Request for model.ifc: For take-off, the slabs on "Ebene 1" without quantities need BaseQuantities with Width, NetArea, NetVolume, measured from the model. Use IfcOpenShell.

First a look at what the model holds.

```python
import ifcopenshell
import ifcopenshell.util.element
import ifcopenshell.util.unit

model = ifcopenshell.open("model.ifc")
print(model.schema)
for unit_type in ("LENGTHUNIT", "AREAUNIT", "VOLUMEUNIT"):
    print(unit_type, ifcopenshell.util.unit.calculate_unit_scale(model, unit_type))
storey = next(s for s in model.by_type("IfcBuildingStorey") if s.Name == "Ebene 1")
slabs = [e for e in ifcopenshell.util.element.get_decomposition(storey) if e.is_a("IfcSlab")]
for e in sorted(slabs, key=lambda e: e.id()):
    print(e.id(), e.is_a(), e.Name, list(ifcopenshell.util.element.get_psets(e, qtos_only=True)), sep=" | ")
```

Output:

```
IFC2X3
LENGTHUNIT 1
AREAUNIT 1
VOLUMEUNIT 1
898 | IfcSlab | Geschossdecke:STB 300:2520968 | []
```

```python
import ifcopenshell
import ifcopenshell.api.pset
import ifcopenshell.geom
import ifcopenshell.util.element
import ifcopenshell.util.shape
import ifcopenshell.util.unit

model = ifcopenshell.open("model.ifc")
unit_scale = ifcopenshell.util.unit.calculate_unit_scale(model)
area_scale = ifcopenshell.util.unit.calculate_unit_scale(model, "AREAUNIT")
volume_scale = ifcopenshell.util.unit.calculate_unit_scale(model, "VOLUMEUNIT")
settings = ifcopenshell.geom.settings()

storey = next(s for s in model.by_type("IfcBuildingStorey") if s.Name == "Ebene 1")
slabs = [e for e in ifcopenshell.util.element.get_decomposition(storey) if e.is_a("IfcSlab")]

for e in sorted(slabs, key=lambda e: e.id()):
    if ifcopenshell.util.element.get_psets(e, qtos_only=True, should_inherit=False):
        continue
    # Geometry comes back in metres, in the element's own axes.
    shape = ifcopenshell.geom.create_shape(settings, e)
    values = {
        "Width": ifcopenshell.util.shape.get_z(shape.geometry) / unit_scale,
        "NetArea": ifcopenshell.util.shape.get_footprint_area(shape.geometry) / area_scale,
        "NetVolume": ifcopenshell.util.shape.get_volume(shape.geometry) / volume_scale,
    }
    qto = ifcopenshell.api.pset.add_qto(model, product=e, name="BaseQuantities")
    ifcopenshell.api.pset.edit_qto(model, qto=qto, properties=values)
    print(e.id(), {k: round(v, 3) for k, v in values.items()})

model.write("model_rev.ifc")
```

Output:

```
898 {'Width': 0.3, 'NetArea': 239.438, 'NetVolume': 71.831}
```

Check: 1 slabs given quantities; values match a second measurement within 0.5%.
